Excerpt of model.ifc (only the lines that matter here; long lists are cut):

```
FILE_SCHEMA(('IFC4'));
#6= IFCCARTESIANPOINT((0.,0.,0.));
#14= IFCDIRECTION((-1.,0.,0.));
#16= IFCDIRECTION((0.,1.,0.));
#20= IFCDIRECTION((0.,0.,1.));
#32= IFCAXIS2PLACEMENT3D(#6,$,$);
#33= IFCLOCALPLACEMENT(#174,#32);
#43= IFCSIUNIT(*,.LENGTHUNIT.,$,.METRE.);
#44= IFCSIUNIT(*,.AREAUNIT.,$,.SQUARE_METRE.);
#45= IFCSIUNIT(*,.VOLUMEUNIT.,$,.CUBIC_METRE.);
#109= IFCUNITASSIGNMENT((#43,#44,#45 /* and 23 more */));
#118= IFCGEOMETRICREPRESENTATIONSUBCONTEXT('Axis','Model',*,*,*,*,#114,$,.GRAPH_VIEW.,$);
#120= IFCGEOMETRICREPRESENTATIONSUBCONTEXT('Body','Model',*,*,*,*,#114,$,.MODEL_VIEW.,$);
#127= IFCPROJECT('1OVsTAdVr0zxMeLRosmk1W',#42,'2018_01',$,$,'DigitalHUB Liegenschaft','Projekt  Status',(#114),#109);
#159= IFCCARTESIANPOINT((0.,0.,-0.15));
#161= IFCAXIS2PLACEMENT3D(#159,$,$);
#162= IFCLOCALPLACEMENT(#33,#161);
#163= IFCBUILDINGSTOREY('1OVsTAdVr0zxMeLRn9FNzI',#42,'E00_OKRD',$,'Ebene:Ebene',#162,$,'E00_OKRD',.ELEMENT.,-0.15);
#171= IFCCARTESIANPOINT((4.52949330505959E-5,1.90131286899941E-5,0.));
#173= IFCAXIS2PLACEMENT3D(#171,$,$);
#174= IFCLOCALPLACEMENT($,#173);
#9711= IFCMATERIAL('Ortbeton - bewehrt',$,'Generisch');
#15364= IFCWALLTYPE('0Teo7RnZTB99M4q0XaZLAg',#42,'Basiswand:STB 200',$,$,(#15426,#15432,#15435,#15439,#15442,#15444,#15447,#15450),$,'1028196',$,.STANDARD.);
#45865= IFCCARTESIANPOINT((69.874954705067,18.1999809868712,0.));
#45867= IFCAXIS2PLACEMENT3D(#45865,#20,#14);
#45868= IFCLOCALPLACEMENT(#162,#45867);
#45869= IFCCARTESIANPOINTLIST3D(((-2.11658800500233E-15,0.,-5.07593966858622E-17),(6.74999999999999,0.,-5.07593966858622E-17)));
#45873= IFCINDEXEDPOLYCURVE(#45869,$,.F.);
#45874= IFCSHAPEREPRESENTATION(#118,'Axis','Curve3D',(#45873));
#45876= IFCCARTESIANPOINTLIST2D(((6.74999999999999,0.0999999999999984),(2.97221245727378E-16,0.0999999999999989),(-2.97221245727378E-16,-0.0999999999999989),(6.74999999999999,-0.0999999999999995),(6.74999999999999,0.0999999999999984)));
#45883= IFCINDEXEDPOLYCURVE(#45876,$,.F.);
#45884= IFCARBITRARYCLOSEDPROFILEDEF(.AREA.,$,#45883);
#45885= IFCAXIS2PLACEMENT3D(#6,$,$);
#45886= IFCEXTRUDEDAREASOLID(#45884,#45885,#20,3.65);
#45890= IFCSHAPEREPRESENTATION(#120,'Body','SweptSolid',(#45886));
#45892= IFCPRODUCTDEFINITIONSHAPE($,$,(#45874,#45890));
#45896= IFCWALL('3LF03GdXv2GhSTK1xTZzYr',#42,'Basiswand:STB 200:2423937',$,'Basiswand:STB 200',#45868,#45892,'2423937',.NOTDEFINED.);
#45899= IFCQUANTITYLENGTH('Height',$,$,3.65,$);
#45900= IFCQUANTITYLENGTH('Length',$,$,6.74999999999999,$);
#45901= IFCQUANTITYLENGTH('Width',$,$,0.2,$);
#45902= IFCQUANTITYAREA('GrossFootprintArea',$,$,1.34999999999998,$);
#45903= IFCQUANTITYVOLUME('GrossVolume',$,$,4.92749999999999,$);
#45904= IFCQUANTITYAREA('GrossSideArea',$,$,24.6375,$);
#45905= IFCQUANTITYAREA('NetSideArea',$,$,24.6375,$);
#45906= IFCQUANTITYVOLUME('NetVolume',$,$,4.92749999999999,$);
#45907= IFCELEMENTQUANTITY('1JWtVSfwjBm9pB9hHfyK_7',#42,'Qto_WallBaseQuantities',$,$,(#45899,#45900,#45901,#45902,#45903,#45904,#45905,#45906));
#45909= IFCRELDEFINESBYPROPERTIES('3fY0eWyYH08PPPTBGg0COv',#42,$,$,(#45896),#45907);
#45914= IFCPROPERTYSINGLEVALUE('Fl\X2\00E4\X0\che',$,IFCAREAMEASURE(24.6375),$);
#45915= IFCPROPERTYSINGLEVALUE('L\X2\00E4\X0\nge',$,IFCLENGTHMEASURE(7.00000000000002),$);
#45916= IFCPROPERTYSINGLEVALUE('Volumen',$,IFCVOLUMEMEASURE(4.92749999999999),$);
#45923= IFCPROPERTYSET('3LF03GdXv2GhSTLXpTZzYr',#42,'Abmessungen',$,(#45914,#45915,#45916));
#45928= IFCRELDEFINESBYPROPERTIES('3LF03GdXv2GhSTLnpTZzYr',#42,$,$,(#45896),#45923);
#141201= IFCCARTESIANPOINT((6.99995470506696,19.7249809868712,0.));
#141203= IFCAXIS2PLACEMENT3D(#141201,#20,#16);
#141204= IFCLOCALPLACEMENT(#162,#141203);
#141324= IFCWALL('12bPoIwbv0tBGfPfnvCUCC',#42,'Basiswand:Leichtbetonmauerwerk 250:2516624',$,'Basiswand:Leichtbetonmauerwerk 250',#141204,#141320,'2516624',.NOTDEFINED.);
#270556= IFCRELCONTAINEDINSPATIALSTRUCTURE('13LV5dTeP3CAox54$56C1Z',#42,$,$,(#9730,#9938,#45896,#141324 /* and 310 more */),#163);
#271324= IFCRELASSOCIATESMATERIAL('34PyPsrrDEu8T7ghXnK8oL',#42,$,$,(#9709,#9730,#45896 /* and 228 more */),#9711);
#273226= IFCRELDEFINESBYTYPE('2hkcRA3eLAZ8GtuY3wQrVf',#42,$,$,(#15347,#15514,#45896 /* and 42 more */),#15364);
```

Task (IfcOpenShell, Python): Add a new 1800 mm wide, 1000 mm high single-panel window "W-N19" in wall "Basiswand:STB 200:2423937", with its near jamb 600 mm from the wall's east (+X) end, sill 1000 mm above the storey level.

```python
import numpy as np
import ifcopenshell
import ifcopenshell.api.feature
import ifcopenshell.api.geometry
import ifcopenshell.api.pset
import ifcopenshell.api.root
import ifcopenshell.api.spatial
import ifcopenshell.geom
import ifcopenshell.util.element
import ifcopenshell.util.placement
import ifcopenshell.util.representation
import ifcopenshell.util.shape
import ifcopenshell.util.unit

model = ifcopenshell.open("model.ifc")
unit_scale = ifcopenshell.util.unit.calculate_unit_scale(model)
area_scale = ifcopenshell.util.unit.calculate_unit_scale(model, "AREAUNIT")
volume_scale = ifcopenshell.util.unit.calculate_unit_scale(model, "VOLUMEUNIT")
settings = ifcopenshell.geom.settings()


def volume(element):
    """Net volume in cubic metres, openings subtracted."""
    shape = ifcopenshell.geom.create_shape(settings, element)
    return ifcopenshell.util.shape.get_volume(shape.geometry)


wall = model.by_guid("3LF03GdXv2GhSTK1xTZzYr")
storey = ifcopenshell.util.element.get_container(wall, ifc_class="IfcBuildingStorey")
context = ifcopenshell.util.representation.get_context(model, "Model", "Body", "MODEL_VIEW")
before = volume(wall)

width, height, from_end, sill = 1.8, 1, 0.6, 1  # metres

# The wall runs along its own X axis, and the end named is its -X end.
wall_shape = ifcopenshell.geom.create_shape(settings, wall)
x, y, z = ifcopenshell.util.shape.get_vertices(wall_shape.geometry).T
start = x.min() + from_end
face, thickness = float(y.min()), float(y.max() - y.min())
wall_matrix = ifcopenshell.util.placement.get_local_placement(wall.ObjectPlacement)
level = ifcopenshell.util.placement.get_local_placement(storey.ObjectPlacement)[2, 3]


def in_wall(x, y):
    """Placement at x, y metres in the wall's axes, at sill height."""
    matrix = wall_matrix.copy()
    matrix[:, 3] = wall_matrix @ np.array([x / unit_scale, y / unit_scale, 0.0, 1.0])
    matrix[2, 3] = level + sill / unit_scale
    return matrix


# Opening: a box that overshoots both wall faces by 50 mm.
opening = ifcopenshell.api.root.create_entity(model, ifc_class="IfcOpeningElement", predefined_type="OPENING")
box = ifcopenshell.api.geometry.add_wall_representation(
    model, context=context, length=width, height=height, thickness=thickness + 0.1
)
ifcopenshell.api.geometry.assign_representation(model, product=opening, representation=box)
ifcopenshell.api.geometry.edit_object_placement(model, product=opening, matrix=in_wall(start, face - 0.05), is_si=False)
ifcopenshell.api.feature.add_feature(model, feature=opening, element=wall)

window = ifcopenshell.api.root.create_entity(model, ifc_class="IfcWindow", name="W-N19", predefined_type="WINDOW")
window.OverallWidth, window.OverallHeight = width / unit_scale, height / unit_scale
window.PartitioningType = "SINGLE_PANEL"
body = ifcopenshell.api.geometry.add_window_representation(
    model,
    context=context,
    overall_width=window.OverallWidth,
    overall_height=window.OverallHeight,
    partition_type="SINGLE_PANEL",
)
ifcopenshell.api.geometry.assign_representation(model, product=window, representation=body)
ifcopenshell.api.spatial.assign_container(model, products=[window], relating_structure=storey)
ifcopenshell.api.feature.add_filling(model, opening=opening, element=window)

# Centre the window in the wall's thickness.
ifcopenshell.api.geometry.edit_object_placement(model, product=window, matrix=in_wall(start, face), is_si=False)
window_shape = ifcopenshell.geom.create_shape(settings, window)
depth = ifcopenshell.util.shape.get_vertices(window_shape.geometry)[:, 1]
offset = face + thickness / 2 - (depth.min() + depth.max()) / 2
ifcopenshell.api.geometry.edit_object_placement(model, product=window, matrix=in_wall(start, offset), is_si=False)

after = volume(wall)

# Update the wall's stored quantities.
qto = model.by_id(ifcopenshell.util.element.get_pset(wall, "Qto_WallBaseQuantities", should_inherit=False)["id"])
ifcopenshell.api.pset.edit_qto(model, qto=qto, properties={
    "NetSideArea": after / thickness / area_scale,
    "NetVolume": after / volume_scale,
})
pset = model.by_id(ifcopenshell.util.element.get_pset(wall, "Abmessungen", should_inherit=False)["id"])
ifcopenshell.api.pset.edit_pset(model, pset=pset, properties={
    "Fläche": model.create_entity("IfcAreaMeasure", after / thickness / area_scale),
    "Volumen": model.create_entity("IfcVolumeMeasure", after / volume_scale),
})

print(f"wall volume {before:.3f} -> {after:.3f} m3")

model.write("model-out.ifc")
```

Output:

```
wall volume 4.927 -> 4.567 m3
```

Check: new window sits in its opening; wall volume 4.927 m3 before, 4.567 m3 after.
